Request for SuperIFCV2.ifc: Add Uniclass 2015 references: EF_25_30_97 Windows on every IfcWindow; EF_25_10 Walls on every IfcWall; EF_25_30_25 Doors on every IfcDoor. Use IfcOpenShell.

First a look at what the model holds.

```python
import ifcopenshell

model = ifcopenshell.open("SuperIFCV2.ifc")
print(model.schema)
print("classifications:", [c.Name for c in model.by_type("IfcClassification")])
for ifc_class in ("IfcDoor", "IfcRoof", "IfcStair", "IfcWall", "IfcWindow"):
    print(ifc_class, len(model.by_type(ifc_class)))
```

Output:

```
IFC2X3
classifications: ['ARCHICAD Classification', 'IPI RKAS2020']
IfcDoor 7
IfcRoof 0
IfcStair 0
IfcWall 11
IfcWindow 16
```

```python
import ifcopenshell
import ifcopenshell.api.classification

model = ifcopenshell.open("SuperIFCV2.ifc")

# IFC2X3 requires Source and Edition and has no link from the project to the system.
system = model.create_entity("IfcClassification", Source="NBS", Edition="2015", Name="Uniclass 2015")

codes = {
    "IfcWindow": ("EF_25_30_97", "Windows"),
    "IfcWall": ("EF_25_10", "Walls"),
    "IfcDoor": ("EF_25_30_25", "Doors"),
}
for ifc_class, (code, name) in codes.items():
    products = model.by_type(ifc_class)
    ifcopenshell.api.classification.add_reference(
        model, products=products, classification=system, identification=code, name=name
    )
    print(code, len(products))

model.write("SuperIFCV2-out.ifc")
```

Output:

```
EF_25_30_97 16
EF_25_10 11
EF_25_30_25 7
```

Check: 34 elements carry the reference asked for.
